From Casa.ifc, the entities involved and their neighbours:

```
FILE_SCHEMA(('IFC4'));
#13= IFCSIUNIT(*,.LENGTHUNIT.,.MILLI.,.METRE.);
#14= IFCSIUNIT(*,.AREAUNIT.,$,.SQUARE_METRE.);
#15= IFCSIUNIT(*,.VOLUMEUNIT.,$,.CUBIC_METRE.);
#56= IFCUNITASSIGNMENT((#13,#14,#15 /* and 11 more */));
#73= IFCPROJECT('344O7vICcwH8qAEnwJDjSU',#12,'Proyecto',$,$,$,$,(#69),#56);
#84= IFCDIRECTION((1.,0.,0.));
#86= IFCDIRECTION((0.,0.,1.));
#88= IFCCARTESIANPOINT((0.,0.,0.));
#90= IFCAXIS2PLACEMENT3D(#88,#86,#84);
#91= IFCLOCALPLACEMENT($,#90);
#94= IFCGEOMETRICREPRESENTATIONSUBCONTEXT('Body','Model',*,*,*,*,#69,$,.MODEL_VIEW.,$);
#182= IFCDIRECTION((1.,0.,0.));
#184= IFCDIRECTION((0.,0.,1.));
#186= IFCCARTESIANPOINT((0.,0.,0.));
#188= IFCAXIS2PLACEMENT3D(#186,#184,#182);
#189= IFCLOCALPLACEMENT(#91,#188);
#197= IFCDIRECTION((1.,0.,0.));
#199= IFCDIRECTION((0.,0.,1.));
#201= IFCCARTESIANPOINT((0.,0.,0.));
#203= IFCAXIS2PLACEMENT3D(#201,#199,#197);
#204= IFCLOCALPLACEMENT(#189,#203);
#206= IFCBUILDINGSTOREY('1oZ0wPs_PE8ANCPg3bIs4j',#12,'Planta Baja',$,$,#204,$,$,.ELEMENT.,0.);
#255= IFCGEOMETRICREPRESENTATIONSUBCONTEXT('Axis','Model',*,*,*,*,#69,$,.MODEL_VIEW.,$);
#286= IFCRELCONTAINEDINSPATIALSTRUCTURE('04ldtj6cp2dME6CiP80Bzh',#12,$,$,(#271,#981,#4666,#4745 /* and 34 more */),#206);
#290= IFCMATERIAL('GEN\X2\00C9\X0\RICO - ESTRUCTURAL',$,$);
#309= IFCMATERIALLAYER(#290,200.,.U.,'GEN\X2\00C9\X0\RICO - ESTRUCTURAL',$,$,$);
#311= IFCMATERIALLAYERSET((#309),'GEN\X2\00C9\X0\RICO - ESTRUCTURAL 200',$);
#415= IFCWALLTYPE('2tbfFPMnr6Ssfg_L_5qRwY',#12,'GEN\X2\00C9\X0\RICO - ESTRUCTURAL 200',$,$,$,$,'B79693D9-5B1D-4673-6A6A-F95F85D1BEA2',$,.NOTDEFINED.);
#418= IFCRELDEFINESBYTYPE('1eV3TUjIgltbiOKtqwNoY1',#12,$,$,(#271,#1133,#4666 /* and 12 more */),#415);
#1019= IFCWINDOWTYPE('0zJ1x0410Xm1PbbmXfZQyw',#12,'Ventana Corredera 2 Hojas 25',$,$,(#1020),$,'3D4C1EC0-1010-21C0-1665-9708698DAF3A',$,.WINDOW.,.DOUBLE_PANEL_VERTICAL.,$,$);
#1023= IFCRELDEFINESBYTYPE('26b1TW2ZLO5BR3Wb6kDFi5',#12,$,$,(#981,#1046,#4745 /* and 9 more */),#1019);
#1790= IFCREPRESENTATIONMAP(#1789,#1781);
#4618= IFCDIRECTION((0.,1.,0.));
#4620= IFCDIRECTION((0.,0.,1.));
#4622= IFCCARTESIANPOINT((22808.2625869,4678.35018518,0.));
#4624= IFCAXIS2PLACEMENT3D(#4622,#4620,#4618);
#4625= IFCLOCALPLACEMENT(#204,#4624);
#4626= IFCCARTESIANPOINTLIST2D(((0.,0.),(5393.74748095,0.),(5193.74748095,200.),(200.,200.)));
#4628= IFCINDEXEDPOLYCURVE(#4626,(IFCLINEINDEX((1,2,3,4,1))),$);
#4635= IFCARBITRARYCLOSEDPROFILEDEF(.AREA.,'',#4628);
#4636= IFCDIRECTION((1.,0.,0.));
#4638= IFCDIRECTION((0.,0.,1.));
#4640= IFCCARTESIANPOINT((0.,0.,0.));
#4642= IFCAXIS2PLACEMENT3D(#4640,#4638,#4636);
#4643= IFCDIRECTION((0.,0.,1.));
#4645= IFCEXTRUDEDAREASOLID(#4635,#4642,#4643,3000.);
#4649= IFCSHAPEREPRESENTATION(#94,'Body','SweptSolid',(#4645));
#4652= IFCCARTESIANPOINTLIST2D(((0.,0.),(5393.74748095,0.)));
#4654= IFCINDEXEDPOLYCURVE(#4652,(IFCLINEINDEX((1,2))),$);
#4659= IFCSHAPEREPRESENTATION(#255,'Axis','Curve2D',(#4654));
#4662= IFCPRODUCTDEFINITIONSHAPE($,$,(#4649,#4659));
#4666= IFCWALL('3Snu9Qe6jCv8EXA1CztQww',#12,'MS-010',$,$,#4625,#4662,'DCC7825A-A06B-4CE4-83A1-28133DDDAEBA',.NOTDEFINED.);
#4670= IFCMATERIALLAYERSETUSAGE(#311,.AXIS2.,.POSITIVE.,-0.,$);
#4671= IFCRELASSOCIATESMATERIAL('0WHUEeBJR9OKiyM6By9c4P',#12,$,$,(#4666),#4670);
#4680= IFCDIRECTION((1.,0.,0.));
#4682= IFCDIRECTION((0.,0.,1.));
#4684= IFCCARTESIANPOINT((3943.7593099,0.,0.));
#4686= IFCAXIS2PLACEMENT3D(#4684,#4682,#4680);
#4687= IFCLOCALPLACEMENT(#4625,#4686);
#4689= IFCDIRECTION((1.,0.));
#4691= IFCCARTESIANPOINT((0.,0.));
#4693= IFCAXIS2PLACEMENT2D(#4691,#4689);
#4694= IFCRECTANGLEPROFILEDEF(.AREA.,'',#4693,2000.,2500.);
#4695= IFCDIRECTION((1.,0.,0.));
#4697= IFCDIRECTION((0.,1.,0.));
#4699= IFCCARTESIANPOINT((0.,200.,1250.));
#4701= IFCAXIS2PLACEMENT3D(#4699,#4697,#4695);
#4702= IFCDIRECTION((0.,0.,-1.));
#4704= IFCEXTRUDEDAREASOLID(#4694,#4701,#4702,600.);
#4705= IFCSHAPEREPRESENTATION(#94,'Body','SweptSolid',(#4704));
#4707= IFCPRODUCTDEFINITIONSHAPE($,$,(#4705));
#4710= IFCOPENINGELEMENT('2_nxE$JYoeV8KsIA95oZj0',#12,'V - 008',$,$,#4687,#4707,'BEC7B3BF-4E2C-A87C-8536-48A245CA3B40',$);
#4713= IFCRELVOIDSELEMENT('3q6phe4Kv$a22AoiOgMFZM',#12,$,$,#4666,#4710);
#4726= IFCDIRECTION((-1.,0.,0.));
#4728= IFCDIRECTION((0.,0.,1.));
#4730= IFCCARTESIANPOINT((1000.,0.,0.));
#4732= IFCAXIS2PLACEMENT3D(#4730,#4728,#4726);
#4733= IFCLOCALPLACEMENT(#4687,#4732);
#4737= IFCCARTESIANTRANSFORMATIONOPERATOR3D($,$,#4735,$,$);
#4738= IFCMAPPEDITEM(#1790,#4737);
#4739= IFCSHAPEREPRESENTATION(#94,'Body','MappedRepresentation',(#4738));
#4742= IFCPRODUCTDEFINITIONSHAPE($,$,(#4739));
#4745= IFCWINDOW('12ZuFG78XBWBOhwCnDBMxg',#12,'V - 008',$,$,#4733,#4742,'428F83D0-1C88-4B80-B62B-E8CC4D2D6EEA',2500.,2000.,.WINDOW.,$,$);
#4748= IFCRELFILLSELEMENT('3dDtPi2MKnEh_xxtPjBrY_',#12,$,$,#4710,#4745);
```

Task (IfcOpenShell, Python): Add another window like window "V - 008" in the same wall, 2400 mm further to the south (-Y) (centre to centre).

```python
import ifcopenshell
import ifcopenshell.api.feature
import ifcopenshell.api.geometry
import ifcopenshell.api.root
import ifcopenshell.geom
import ifcopenshell.util.element
import ifcopenshell.util.placement
import ifcopenshell.util.shape

model = ifcopenshell.open("Casa.ifc")
settings = ifcopenshell.geom.settings()


def volume(element):
    """Net volume in cubic metres, openings subtracted."""
    shape = ifcopenshell.geom.create_shape(settings, element)
    return ifcopenshell.util.shape.get_volume(shape.geometry)


def reuse_history(source, copy):
    """copy_class also copies each property set's owner history, people and application; keep the originals."""
    for rel in copy.IsDefinedBy:
        if rel.is_a("IfcRelDefinesByProperties") and (history := rel.RelatingPropertyDefinition.OwnerHistory):
            rel.RelatingPropertyDefinition.OwnerHistory = source.OwnerHistory
            ifcopenshell.util.element.remove_deep2(model, history)


window = model.by_id(4745)
opening = window.FillsVoids[0].RelatingOpeningElement
wall = opening.VoidsElements[0].RelatingBuildingElement
before = volume(wall)
shift = ifcopenshell.util.placement.get_local_placement(wall.ObjectPlacement)[:3, 0] * -2400.0

# copy_class copies the void relationship, type, container and properties, but no geometry.
new_opening = ifcopenshell.api.root.copy_class(model, product=opening)
new_opening.Representation = ifcopenshell.util.element.copy_deep(
    model, opening.Representation, exclude=["IfcGeometricRepresentationContext", "IfcRepresentationMap"]
)
new_opening.Tag = None
new_window = ifcopenshell.api.root.copy_class(model, product=window)
new_window.Representation = ifcopenshell.util.element.copy_deep(
    model, window.Representation, exclude=["IfcGeometricRepresentationContext", "IfcRepresentationMap"]
)
new_window.Tag = None
reuse_history(window, new_window)
ifcopenshell.api.feature.add_filling(model, opening=new_opening, element=new_window)

for old, new in ((opening, new_opening), (window, new_window)):
    matrix = ifcopenshell.util.placement.get_local_placement(old.ObjectPlacement)
    matrix[:3, 3] += shift
    ifcopenshell.api.geometry.edit_object_placement(model, product=new, matrix=matrix, is_si=False)

after = volume(wall)

print(f"wall volume {before:.3f} -> {after:.3f} m3")

model.write("Casa_v2.ifc")
```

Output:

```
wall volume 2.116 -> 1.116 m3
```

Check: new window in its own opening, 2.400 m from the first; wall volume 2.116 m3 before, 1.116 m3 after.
